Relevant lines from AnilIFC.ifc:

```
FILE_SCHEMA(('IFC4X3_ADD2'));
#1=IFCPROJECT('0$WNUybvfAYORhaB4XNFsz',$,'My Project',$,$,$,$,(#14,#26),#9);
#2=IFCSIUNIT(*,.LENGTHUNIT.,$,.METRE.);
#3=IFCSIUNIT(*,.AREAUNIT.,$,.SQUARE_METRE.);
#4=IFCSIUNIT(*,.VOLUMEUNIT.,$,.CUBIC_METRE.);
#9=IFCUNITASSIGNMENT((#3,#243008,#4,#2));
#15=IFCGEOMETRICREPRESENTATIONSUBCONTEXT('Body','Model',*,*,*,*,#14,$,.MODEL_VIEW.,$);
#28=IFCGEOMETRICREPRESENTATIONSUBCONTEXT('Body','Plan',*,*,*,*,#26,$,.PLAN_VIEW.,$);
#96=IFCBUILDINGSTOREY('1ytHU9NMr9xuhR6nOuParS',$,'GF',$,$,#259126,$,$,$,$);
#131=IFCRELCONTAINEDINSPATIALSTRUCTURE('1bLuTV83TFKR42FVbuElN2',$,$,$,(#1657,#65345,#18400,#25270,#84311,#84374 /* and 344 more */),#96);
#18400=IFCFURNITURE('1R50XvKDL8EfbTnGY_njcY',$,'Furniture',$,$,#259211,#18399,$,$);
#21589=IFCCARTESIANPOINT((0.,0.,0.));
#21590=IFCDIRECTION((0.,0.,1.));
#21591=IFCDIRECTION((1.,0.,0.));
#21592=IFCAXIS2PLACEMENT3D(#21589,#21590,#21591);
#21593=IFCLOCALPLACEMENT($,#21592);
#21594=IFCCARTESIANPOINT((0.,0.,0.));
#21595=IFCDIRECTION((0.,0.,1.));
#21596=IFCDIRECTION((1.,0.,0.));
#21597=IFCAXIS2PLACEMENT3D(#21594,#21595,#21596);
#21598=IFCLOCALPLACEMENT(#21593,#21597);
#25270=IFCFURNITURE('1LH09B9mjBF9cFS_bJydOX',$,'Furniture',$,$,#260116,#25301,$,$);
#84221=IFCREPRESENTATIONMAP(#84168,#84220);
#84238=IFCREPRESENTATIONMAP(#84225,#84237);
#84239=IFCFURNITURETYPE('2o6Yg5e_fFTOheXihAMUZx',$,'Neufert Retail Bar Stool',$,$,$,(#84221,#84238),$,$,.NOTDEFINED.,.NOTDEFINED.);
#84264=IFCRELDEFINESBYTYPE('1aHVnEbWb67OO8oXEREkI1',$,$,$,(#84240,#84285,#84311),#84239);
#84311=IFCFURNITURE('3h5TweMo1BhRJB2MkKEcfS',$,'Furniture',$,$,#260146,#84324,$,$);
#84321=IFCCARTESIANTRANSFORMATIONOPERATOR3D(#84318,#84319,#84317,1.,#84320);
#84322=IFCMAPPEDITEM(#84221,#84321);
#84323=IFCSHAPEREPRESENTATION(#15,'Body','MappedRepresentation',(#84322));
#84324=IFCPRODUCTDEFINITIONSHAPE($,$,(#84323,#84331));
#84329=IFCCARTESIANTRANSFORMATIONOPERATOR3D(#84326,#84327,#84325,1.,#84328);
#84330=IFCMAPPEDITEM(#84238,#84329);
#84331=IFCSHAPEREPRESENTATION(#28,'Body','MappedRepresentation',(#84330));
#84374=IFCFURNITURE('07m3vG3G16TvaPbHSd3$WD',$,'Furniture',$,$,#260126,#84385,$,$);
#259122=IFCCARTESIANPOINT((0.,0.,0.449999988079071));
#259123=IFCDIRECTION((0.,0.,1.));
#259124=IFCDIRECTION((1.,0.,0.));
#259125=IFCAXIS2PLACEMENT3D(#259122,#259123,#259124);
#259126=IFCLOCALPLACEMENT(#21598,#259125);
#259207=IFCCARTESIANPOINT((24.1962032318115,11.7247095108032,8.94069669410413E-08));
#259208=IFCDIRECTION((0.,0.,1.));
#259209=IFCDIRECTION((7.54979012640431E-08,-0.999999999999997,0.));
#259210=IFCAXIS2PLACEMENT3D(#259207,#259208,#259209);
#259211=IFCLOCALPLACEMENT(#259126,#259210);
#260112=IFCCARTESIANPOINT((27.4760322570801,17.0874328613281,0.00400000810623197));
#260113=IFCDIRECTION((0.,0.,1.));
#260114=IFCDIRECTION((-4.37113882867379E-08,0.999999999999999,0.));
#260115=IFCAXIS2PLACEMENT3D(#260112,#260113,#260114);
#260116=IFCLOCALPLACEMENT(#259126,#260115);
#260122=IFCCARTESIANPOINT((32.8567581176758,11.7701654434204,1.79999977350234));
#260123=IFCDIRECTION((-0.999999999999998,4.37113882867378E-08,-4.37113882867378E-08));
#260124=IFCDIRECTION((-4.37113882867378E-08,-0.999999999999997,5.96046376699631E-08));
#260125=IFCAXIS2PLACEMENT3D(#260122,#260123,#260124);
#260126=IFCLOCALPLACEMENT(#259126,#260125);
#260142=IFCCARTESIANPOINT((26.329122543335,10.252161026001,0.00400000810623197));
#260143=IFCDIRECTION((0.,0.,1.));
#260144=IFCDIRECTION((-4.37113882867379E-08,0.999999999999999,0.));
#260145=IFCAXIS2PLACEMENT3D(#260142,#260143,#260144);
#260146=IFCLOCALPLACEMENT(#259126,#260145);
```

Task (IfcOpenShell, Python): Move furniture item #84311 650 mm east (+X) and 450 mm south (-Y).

```python
import ifcopenshell
import ifcopenshell.api.geometry
import ifcopenshell.util.placement
import ifcopenshell.util.unit

model = ifcopenshell.open("AnilIFC.ifc")
unit_scale = ifcopenshell.util.unit.calculate_unit_scale(model)

item = model.by_id(84311)
matrix = ifcopenshell.util.placement.get_local_placement(item.ObjectPlacement)
matrix[0, 3] += 0.65 / unit_scale
matrix[1, 3] -= 0.45 / unit_scale
ifcopenshell.api.geometry.edit_object_placement(model, product=item, matrix=matrix, is_si=False)

print(ifcopenshell.util.placement.get_local_placement(item.ObjectPlacement).round(3) + 0.0)

model.write("AnilIFC_edited.ifc")
```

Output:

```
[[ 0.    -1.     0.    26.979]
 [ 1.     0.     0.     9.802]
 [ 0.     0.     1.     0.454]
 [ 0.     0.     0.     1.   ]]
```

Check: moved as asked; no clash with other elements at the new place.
